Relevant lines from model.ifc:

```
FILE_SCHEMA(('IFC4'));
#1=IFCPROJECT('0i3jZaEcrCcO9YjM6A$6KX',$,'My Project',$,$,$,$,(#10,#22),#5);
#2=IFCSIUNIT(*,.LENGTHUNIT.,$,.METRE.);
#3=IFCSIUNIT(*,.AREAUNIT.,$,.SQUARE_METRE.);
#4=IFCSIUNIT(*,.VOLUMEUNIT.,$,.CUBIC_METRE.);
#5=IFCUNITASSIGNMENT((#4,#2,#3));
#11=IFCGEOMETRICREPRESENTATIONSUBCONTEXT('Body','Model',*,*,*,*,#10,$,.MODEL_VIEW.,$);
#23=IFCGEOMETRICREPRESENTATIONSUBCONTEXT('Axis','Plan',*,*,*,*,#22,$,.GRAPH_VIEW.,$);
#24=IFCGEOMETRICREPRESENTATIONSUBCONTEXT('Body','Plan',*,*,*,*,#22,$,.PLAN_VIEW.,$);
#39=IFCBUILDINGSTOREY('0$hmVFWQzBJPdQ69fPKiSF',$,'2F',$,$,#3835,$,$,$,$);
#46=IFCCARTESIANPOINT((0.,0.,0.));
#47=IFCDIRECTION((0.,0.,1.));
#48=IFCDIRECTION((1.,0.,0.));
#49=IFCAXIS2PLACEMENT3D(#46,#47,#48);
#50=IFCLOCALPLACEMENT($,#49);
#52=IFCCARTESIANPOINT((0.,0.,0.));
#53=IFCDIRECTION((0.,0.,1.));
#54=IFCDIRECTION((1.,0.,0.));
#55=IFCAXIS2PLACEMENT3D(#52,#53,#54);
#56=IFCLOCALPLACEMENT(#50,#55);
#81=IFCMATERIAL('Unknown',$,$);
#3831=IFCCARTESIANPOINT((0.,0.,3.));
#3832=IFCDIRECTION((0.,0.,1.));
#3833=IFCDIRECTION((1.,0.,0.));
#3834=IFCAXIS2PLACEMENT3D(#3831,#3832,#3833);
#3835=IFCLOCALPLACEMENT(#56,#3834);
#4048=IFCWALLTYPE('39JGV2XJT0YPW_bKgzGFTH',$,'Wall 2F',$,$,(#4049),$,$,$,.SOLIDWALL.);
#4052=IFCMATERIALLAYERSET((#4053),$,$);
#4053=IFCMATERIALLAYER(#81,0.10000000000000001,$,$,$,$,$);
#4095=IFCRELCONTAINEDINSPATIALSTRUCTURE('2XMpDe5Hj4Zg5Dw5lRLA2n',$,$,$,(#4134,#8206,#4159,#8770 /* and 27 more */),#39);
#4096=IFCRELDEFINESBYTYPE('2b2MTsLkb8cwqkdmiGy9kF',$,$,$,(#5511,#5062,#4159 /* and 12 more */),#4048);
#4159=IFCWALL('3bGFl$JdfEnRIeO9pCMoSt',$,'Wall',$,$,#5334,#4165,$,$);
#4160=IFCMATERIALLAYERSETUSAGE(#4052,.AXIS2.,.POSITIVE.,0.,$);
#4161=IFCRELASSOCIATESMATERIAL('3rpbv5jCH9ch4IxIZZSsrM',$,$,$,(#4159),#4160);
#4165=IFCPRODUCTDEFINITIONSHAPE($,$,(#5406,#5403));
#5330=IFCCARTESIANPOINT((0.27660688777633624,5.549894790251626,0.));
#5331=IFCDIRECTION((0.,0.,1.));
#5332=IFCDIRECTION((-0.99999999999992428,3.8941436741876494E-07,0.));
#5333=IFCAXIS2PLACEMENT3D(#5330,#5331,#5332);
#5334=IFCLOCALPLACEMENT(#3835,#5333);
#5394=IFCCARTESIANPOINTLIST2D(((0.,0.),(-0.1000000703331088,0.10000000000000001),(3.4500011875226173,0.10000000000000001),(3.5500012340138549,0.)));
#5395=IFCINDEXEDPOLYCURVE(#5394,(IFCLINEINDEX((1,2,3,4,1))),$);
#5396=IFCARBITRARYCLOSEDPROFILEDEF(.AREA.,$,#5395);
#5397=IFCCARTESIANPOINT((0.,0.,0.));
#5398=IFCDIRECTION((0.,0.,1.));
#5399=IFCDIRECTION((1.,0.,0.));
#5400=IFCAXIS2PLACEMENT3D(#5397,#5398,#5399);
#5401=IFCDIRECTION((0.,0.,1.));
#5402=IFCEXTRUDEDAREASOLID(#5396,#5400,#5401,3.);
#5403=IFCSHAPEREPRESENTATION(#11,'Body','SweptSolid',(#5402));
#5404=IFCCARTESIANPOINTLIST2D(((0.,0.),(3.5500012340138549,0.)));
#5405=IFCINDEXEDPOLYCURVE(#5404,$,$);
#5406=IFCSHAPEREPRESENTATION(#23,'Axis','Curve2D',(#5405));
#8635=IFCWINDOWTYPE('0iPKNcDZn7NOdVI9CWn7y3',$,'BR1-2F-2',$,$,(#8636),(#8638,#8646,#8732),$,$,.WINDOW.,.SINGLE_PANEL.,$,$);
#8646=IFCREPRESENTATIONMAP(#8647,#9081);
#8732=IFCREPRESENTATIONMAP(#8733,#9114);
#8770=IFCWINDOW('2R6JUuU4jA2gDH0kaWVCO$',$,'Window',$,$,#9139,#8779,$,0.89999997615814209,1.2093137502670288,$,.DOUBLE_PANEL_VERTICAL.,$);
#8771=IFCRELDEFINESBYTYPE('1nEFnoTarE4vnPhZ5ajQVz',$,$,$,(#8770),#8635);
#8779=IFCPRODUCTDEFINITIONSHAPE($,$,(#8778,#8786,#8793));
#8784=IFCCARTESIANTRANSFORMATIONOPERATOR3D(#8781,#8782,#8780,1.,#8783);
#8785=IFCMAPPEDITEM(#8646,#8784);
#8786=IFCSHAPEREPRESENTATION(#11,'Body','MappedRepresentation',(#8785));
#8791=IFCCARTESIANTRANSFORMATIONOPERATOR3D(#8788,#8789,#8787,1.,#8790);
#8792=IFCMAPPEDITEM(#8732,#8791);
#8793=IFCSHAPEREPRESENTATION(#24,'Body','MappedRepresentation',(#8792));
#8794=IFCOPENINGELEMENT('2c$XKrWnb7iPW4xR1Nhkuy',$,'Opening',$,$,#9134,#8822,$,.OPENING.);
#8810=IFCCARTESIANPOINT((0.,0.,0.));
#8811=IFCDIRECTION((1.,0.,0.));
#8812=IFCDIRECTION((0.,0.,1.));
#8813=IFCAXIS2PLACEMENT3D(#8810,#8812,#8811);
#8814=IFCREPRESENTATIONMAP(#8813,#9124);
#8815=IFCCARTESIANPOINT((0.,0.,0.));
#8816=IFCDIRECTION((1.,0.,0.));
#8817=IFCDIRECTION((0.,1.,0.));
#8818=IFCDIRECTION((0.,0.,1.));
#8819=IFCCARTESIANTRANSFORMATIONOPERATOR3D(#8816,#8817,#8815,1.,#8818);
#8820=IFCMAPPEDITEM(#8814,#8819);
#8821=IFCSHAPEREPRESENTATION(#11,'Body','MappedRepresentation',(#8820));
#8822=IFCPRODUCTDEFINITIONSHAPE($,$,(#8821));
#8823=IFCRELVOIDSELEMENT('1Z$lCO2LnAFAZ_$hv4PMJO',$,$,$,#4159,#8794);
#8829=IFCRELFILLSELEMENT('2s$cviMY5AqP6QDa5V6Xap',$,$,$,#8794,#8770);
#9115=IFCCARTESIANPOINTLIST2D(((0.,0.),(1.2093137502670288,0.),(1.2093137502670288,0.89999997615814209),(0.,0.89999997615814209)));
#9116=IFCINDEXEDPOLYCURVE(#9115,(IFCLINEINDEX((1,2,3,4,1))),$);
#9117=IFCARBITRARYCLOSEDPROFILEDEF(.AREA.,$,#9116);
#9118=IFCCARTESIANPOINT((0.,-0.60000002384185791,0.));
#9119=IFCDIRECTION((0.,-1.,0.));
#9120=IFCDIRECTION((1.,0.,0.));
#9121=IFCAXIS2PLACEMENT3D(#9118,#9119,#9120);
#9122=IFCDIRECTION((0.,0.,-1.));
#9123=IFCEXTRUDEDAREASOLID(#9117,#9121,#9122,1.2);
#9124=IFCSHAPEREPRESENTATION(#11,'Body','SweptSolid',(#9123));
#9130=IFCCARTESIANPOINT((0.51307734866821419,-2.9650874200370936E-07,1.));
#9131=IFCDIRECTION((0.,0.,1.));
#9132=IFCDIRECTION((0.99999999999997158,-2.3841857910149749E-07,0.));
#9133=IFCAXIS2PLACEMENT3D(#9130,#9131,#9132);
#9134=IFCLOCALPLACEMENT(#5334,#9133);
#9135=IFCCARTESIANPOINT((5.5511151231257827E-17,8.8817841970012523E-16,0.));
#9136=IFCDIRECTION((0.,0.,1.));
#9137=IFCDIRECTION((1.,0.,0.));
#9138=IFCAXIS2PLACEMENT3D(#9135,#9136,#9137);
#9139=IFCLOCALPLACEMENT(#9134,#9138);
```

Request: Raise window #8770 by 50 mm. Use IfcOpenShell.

```python
import numpy as np
import ifcopenshell
import ifcopenshell.api.geometry
import ifcopenshell.util.placement
import ifcopenshell.util.unit

model = ifcopenshell.open("model.ifc")
unit_scale = ifcopenshell.util.unit.calculate_unit_scale(model)

window = model.by_guid("2R6JUuU4jA2gDH0kaWVCO$")
opening = window.FillsVoids[0].RelatingOpeningElement
dz = 0.05

shift = np.array([0.0, 0.0, dz])
# The window is placed relative to its opening, so it follows when the opening moves.
matrix = ifcopenshell.util.placement.get_local_placement(opening.ObjectPlacement)
matrix[:3, 3] += shift
ifcopenshell.api.geometry.edit_object_placement(
    model, product=opening, matrix=matrix, is_si=False, should_transform_children=True
)

print(f"moved by {dz * unit_scale:+.3f} m")

model.write("model_rev.ifc")
```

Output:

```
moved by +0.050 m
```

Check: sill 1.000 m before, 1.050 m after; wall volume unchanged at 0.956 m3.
